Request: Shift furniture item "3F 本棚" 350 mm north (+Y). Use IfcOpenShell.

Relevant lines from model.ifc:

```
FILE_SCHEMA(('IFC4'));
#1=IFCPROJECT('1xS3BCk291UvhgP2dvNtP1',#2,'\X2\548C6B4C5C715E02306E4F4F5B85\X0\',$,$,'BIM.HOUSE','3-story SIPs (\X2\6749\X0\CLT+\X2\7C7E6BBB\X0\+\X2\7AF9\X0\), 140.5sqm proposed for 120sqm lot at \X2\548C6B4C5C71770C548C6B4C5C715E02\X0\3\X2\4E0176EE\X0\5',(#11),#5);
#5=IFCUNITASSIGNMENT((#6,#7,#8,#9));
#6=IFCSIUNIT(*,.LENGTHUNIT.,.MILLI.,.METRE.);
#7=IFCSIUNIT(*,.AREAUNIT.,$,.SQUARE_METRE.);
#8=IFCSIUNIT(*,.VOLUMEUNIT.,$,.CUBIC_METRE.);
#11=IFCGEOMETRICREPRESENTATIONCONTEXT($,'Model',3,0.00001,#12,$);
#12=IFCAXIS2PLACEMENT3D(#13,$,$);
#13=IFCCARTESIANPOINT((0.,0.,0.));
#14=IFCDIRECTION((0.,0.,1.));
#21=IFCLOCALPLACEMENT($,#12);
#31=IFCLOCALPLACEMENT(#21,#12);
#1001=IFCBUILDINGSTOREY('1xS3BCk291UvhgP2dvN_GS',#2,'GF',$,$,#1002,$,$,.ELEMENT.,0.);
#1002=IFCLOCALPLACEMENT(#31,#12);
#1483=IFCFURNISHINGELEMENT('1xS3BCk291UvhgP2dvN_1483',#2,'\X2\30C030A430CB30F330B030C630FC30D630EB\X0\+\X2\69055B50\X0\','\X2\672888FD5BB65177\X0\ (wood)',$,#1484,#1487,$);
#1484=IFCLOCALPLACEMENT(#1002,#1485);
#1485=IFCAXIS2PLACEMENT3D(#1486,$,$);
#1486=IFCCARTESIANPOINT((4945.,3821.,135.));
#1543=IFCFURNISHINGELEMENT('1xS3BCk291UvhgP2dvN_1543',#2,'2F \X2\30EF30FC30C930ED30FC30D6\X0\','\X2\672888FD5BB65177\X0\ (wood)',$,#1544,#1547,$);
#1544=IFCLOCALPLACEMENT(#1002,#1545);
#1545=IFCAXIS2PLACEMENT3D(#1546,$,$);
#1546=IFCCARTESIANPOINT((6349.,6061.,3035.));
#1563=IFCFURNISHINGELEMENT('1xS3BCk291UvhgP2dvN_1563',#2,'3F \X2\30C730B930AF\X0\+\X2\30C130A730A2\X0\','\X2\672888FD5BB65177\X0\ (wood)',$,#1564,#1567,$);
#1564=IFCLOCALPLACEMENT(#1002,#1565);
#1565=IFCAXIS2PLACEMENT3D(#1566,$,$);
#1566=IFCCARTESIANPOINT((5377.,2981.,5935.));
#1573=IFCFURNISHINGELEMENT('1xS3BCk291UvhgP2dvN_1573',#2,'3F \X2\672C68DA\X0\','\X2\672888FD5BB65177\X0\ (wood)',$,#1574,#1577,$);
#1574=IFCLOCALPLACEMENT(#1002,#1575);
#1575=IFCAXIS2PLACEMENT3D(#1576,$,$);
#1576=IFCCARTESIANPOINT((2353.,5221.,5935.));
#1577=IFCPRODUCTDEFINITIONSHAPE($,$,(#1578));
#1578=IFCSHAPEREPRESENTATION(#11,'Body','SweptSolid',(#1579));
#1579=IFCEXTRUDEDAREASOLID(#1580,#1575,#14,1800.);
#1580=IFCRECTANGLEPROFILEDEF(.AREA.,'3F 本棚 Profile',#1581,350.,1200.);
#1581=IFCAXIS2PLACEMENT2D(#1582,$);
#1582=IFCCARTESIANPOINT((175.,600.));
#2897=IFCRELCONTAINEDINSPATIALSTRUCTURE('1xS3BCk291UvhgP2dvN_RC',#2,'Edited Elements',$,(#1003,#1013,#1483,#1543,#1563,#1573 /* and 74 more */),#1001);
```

```python
import ifcopenshell
import ifcopenshell.api.geometry
import ifcopenshell.util.placement

model = ifcopenshell.open("model.ifc")

item = model.by_guid("1xS3BCk291UvhgP2dvN_1573")
matrix = ifcopenshell.util.placement.get_local_placement(item.ObjectPlacement)
matrix[1, 3] += 350.0
ifcopenshell.api.geometry.edit_object_placement(model, product=item, matrix=matrix, is_si=False)

print(ifcopenshell.util.placement.get_local_placement(item.ObjectPlacement).round(3) + 0.0)

model.write("model_rev.ifc")
```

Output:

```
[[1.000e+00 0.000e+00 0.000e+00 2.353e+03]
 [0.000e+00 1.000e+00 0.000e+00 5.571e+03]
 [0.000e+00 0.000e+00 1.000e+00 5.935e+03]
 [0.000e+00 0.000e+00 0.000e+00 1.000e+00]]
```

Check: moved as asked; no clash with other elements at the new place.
